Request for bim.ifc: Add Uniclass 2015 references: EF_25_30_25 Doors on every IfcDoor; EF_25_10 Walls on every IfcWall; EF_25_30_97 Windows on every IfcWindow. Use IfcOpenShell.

First a look at what the model holds.

```python
import ifcopenshell

model = ifcopenshell.open("bim.ifc")
print(model.schema)
print("classifications:", [c.Name for c in model.by_type("IfcClassification")])
for ifc_class in ("IfcDoor", "IfcRoof", "IfcStair", "IfcWall", "IfcWindow"):
    print(ifc_class, len(model.by_type(ifc_class)))
```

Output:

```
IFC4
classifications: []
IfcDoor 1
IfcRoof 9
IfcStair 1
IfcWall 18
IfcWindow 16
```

```python
import ifcopenshell
import ifcopenshell.api.classification

model = ifcopenshell.open("bim.ifc")

system = ifcopenshell.api.classification.add_classification(model, classification="Uniclass 2015")

codes = {
    "IfcDoor": ("EF_25_30_25", "Doors"),
    "IfcWall": ("EF_25_10", "Walls"),
    "IfcWindow": ("EF_25_30_97", "Windows"),
}
for ifc_class, (code, name) in codes.items():
    products = model.by_type(ifc_class)
    ifcopenshell.api.classification.add_reference(
        model, products=products, classification=system, identification=code, name=name
    )
    print(code, len(products))

model.write("bim-out.ifc")
```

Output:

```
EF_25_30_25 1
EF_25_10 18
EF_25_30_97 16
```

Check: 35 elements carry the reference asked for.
